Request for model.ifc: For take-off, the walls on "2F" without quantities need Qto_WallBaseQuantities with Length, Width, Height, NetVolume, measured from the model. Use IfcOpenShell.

First a look at what the model holds.

```python
import ifcopenshell
import ifcopenshell.util.element
import ifcopenshell.util.unit

model = ifcopenshell.open("model.ifc")
print(model.schema)
for unit_type in ("LENGTHUNIT", "AREAUNIT", "VOLUMEUNIT"):
    print(unit_type, ifcopenshell.util.unit.calculate_unit_scale(model, unit_type))
storey = next(s for s in model.by_type("IfcBuildingStorey") if s.Name == "2F")
walls = [e for e in ifcopenshell.util.element.get_decomposition(storey) if e.is_a("IfcWall")]
for e in sorted(walls, key=lambda e: e.id()):
    print(e.id(), e.is_a(), e.Name, list(ifcopenshell.util.element.get_psets(e, qtos_only=True)), sep=" | ")
```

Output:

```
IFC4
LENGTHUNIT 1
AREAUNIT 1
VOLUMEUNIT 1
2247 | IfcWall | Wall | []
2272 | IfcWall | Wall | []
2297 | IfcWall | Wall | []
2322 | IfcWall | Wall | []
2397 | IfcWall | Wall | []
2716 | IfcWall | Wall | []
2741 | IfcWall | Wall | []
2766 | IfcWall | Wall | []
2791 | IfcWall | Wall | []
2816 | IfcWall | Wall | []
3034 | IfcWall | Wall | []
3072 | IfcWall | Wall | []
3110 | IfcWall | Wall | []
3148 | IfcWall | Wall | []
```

```python
import ifcopenshell
import ifcopenshell.api.pset
import ifcopenshell.geom
import ifcopenshell.util.element
import ifcopenshell.util.shape
import ifcopenshell.util.unit

model = ifcopenshell.open("model.ifc")
unit_scale = ifcopenshell.util.unit.calculate_unit_scale(model)
volume_scale = ifcopenshell.util.unit.calculate_unit_scale(model, "VOLUMEUNIT")
settings = ifcopenshell.geom.settings()

storey = next(s for s in model.by_type("IfcBuildingStorey") if s.Name == "2F")
walls = [e for e in ifcopenshell.util.element.get_decomposition(storey) if e.is_a("IfcWall")]

for e in sorted(walls, key=lambda e: e.id()):
    if ifcopenshell.util.element.get_psets(e, qtos_only=True, should_inherit=False):
        continue
    # Geometry comes back in metres, in the element's own axes.
    shape = ifcopenshell.geom.create_shape(settings, e)
    values = {
        "Length": ifcopenshell.util.shape.get_x(shape.geometry) / unit_scale,
        "Width": ifcopenshell.util.shape.get_y(shape.geometry) / unit_scale,
        "Height": ifcopenshell.util.shape.get_z(shape.geometry) / unit_scale,
        "NetVolume": ifcopenshell.util.shape.get_volume(shape.geometry) / volume_scale,
    }
    qto = ifcopenshell.api.pset.add_qto(model, product=e, name="Qto_WallBaseQuantities")
    ifcopenshell.api.pset.edit_qto(model, qto=qto, properties=values)
    print(e.id(), {k: round(v, 3) for k, v in values.items()})

model.write("model_edited.ifc")
```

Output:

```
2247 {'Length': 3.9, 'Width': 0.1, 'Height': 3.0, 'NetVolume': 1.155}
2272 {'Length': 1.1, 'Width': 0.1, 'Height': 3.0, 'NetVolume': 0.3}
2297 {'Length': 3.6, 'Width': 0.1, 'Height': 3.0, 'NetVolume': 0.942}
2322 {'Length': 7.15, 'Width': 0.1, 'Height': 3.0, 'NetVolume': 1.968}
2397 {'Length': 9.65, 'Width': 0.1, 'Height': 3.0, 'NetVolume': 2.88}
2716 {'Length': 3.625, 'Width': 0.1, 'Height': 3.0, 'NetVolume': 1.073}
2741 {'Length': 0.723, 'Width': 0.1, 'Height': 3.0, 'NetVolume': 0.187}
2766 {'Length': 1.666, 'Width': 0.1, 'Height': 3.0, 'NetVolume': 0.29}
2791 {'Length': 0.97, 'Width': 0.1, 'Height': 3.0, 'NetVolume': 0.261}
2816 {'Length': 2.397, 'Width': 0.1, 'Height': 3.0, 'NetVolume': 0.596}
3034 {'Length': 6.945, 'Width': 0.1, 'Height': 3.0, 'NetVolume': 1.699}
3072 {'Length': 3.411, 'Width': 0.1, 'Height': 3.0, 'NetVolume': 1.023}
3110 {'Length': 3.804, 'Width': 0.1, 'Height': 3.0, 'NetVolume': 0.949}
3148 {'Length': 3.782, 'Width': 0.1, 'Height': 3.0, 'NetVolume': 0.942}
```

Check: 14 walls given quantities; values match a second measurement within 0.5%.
